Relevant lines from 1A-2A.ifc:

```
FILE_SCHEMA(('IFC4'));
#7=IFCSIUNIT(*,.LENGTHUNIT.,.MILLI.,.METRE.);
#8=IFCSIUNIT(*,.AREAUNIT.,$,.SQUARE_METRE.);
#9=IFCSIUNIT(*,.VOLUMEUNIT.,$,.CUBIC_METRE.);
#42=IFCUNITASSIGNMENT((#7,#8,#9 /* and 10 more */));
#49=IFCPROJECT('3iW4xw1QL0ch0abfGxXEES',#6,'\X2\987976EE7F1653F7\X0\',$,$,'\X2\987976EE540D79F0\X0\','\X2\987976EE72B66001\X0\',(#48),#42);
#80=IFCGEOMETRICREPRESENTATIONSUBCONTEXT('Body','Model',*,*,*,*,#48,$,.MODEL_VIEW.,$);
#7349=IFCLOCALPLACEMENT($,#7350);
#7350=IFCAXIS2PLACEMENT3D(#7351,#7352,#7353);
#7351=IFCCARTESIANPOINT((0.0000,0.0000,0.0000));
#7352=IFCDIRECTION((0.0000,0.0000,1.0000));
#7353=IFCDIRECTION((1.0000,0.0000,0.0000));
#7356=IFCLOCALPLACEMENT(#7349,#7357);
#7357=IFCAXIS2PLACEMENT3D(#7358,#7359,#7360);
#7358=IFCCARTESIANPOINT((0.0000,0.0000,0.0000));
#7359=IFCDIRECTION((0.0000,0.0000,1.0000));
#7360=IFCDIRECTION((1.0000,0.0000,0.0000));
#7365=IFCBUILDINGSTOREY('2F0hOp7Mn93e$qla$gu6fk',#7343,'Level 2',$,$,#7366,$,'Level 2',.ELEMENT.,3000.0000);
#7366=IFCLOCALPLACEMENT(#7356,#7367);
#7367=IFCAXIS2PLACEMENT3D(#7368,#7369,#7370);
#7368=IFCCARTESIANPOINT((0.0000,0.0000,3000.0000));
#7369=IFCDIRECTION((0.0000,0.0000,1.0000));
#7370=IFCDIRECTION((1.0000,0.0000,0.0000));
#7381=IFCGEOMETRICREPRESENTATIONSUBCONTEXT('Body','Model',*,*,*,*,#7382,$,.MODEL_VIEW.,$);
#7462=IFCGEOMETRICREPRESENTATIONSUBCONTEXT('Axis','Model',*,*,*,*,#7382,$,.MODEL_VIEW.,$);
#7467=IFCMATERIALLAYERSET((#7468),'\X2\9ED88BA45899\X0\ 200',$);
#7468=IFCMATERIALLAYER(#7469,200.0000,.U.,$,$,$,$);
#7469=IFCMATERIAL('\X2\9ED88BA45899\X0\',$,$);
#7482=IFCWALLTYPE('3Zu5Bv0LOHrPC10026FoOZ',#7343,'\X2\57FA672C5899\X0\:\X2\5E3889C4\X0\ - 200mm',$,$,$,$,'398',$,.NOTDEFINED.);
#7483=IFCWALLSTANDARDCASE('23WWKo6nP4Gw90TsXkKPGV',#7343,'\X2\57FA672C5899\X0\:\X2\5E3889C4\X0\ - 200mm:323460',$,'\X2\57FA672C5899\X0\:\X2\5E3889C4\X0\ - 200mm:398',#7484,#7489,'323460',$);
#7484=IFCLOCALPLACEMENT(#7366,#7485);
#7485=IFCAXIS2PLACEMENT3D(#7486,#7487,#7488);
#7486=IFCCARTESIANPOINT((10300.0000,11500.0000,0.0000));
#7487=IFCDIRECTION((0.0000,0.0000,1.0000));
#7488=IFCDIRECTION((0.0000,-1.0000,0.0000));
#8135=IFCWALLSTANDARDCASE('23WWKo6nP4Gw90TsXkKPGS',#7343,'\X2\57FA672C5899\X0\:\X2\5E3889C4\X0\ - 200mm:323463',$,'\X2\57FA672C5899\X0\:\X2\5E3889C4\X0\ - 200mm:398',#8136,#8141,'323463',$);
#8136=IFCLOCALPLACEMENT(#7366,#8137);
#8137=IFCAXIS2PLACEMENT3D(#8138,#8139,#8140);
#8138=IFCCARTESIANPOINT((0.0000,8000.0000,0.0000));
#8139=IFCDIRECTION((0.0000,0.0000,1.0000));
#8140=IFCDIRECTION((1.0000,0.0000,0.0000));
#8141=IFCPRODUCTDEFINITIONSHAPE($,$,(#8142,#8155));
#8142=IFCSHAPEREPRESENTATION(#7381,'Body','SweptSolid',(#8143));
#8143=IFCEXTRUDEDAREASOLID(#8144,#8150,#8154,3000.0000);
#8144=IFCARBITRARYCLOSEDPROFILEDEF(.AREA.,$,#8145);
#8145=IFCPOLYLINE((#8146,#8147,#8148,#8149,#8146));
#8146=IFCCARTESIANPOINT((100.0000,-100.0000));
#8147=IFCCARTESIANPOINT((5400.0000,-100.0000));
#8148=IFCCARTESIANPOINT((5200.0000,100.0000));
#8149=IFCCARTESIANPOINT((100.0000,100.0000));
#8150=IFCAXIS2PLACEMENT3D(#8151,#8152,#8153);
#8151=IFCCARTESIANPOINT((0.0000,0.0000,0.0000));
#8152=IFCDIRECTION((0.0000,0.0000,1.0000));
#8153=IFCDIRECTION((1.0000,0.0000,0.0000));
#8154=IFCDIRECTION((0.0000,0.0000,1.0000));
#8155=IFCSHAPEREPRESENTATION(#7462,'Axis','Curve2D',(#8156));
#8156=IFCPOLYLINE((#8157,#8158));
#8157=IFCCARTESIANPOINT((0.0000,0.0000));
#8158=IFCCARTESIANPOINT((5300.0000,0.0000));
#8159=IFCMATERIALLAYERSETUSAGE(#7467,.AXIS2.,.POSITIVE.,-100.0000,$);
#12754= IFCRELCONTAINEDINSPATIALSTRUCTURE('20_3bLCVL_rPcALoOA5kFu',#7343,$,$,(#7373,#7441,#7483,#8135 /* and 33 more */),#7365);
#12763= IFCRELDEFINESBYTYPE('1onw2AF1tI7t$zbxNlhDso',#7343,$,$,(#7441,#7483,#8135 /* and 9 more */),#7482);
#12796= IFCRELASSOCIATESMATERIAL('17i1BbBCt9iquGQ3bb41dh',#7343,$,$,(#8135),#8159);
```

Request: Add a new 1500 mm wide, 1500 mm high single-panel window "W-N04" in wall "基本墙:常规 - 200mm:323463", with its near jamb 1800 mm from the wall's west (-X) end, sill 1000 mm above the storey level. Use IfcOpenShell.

```python
import numpy as np
import ifcopenshell
import ifcopenshell.api.feature
import ifcopenshell.api.geometry
import ifcopenshell.api.root
import ifcopenshell.api.spatial
import ifcopenshell.geom
import ifcopenshell.util.element
import ifcopenshell.util.placement
import ifcopenshell.util.representation
import ifcopenshell.util.shape
import ifcopenshell.util.unit

model = ifcopenshell.open("1A-2A.ifc")
unit_scale = ifcopenshell.util.unit.calculate_unit_scale(model)
settings = ifcopenshell.geom.settings()


def volume(element):
    """Net volume in cubic metres, openings subtracted."""
    shape = ifcopenshell.geom.create_shape(settings, element)
    return ifcopenshell.util.shape.get_volume(shape.geometry)


wall = model.by_guid("23WWKo6nP4Gw90TsXkKPGS")
storey = ifcopenshell.util.element.get_container(wall, ifc_class="IfcBuildingStorey")
context = ifcopenshell.util.representation.get_context(model, "Model", "Body", "MODEL_VIEW")
before = volume(wall)

width, height, from_end, sill = 1.5, 1.5, 1.8, 1  # metres

# The wall runs along its own X axis, and the end named is its -X end.
wall_shape = ifcopenshell.geom.create_shape(settings, wall)
x, y, z = ifcopenshell.util.shape.get_vertices(wall_shape.geometry).T
start = x.min() + from_end
face, thickness = float(y.min()), float(y.max() - y.min())
wall_matrix = ifcopenshell.util.placement.get_local_placement(wall.ObjectPlacement)
level = ifcopenshell.util.placement.get_local_placement(storey.ObjectPlacement)[2, 3]


def in_wall(x, y):
    """Placement at x, y metres in the wall's axes, at sill height."""
    matrix = wall_matrix.copy()
    matrix[:, 3] = wall_matrix @ np.array([x / unit_scale, y / unit_scale, 0.0, 1.0])
    matrix[2, 3] = level + sill / unit_scale
    return matrix


# Opening: a box that overshoots both wall faces by 50 mm.
opening = ifcopenshell.api.root.create_entity(model, ifc_class="IfcOpeningElement", predefined_type="OPENING")
box = ifcopenshell.api.geometry.add_wall_representation(
    model, context=context, length=width, height=height, thickness=thickness + 0.1
)
ifcopenshell.api.geometry.assign_representation(model, product=opening, representation=box)
ifcopenshell.api.geometry.edit_object_placement(model, product=opening, matrix=in_wall(start, face - 0.05), is_si=False)
ifcopenshell.api.feature.add_feature(model, feature=opening, element=wall)

window = ifcopenshell.api.root.create_entity(model, ifc_class="IfcWindow", name="W-N04", predefined_type="WINDOW")
window.OverallWidth, window.OverallHeight = width / unit_scale, height / unit_scale
window.PartitioningType = "SINGLE_PANEL"
body = ifcopenshell.api.geometry.add_window_representation(
    model,
    context=context,
    overall_width=window.OverallWidth,
    overall_height=window.OverallHeight,
    partition_type="SINGLE_PANEL",
)
ifcopenshell.api.geometry.assign_representation(model, product=window, representation=body)
ifcopenshell.api.spatial.assign_container(model, products=[window], relating_structure=storey)
ifcopenshell.api.feature.add_filling(model, opening=opening, element=window)

# Centre the window in the wall's thickness.
ifcopenshell.api.geometry.edit_object_placement(model, product=window, matrix=in_wall(start, face), is_si=False)
window_shape = ifcopenshell.geom.create_shape(settings, window)
depth = ifcopenshell.util.shape.get_vertices(window_shape.geometry)[:, 1]
offset = face + thickness / 2 - (depth.min() + depth.max()) / 2
ifcopenshell.api.geometry.edit_object_placement(model, product=window, matrix=in_wall(start, offset), is_si=False)

after = volume(wall)

print(f"wall volume {before:.3f} -> {after:.3f} m3")

model.write("1A-2A_v2.ifc")
```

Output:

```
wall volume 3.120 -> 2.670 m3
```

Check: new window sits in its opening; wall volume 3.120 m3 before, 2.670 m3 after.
